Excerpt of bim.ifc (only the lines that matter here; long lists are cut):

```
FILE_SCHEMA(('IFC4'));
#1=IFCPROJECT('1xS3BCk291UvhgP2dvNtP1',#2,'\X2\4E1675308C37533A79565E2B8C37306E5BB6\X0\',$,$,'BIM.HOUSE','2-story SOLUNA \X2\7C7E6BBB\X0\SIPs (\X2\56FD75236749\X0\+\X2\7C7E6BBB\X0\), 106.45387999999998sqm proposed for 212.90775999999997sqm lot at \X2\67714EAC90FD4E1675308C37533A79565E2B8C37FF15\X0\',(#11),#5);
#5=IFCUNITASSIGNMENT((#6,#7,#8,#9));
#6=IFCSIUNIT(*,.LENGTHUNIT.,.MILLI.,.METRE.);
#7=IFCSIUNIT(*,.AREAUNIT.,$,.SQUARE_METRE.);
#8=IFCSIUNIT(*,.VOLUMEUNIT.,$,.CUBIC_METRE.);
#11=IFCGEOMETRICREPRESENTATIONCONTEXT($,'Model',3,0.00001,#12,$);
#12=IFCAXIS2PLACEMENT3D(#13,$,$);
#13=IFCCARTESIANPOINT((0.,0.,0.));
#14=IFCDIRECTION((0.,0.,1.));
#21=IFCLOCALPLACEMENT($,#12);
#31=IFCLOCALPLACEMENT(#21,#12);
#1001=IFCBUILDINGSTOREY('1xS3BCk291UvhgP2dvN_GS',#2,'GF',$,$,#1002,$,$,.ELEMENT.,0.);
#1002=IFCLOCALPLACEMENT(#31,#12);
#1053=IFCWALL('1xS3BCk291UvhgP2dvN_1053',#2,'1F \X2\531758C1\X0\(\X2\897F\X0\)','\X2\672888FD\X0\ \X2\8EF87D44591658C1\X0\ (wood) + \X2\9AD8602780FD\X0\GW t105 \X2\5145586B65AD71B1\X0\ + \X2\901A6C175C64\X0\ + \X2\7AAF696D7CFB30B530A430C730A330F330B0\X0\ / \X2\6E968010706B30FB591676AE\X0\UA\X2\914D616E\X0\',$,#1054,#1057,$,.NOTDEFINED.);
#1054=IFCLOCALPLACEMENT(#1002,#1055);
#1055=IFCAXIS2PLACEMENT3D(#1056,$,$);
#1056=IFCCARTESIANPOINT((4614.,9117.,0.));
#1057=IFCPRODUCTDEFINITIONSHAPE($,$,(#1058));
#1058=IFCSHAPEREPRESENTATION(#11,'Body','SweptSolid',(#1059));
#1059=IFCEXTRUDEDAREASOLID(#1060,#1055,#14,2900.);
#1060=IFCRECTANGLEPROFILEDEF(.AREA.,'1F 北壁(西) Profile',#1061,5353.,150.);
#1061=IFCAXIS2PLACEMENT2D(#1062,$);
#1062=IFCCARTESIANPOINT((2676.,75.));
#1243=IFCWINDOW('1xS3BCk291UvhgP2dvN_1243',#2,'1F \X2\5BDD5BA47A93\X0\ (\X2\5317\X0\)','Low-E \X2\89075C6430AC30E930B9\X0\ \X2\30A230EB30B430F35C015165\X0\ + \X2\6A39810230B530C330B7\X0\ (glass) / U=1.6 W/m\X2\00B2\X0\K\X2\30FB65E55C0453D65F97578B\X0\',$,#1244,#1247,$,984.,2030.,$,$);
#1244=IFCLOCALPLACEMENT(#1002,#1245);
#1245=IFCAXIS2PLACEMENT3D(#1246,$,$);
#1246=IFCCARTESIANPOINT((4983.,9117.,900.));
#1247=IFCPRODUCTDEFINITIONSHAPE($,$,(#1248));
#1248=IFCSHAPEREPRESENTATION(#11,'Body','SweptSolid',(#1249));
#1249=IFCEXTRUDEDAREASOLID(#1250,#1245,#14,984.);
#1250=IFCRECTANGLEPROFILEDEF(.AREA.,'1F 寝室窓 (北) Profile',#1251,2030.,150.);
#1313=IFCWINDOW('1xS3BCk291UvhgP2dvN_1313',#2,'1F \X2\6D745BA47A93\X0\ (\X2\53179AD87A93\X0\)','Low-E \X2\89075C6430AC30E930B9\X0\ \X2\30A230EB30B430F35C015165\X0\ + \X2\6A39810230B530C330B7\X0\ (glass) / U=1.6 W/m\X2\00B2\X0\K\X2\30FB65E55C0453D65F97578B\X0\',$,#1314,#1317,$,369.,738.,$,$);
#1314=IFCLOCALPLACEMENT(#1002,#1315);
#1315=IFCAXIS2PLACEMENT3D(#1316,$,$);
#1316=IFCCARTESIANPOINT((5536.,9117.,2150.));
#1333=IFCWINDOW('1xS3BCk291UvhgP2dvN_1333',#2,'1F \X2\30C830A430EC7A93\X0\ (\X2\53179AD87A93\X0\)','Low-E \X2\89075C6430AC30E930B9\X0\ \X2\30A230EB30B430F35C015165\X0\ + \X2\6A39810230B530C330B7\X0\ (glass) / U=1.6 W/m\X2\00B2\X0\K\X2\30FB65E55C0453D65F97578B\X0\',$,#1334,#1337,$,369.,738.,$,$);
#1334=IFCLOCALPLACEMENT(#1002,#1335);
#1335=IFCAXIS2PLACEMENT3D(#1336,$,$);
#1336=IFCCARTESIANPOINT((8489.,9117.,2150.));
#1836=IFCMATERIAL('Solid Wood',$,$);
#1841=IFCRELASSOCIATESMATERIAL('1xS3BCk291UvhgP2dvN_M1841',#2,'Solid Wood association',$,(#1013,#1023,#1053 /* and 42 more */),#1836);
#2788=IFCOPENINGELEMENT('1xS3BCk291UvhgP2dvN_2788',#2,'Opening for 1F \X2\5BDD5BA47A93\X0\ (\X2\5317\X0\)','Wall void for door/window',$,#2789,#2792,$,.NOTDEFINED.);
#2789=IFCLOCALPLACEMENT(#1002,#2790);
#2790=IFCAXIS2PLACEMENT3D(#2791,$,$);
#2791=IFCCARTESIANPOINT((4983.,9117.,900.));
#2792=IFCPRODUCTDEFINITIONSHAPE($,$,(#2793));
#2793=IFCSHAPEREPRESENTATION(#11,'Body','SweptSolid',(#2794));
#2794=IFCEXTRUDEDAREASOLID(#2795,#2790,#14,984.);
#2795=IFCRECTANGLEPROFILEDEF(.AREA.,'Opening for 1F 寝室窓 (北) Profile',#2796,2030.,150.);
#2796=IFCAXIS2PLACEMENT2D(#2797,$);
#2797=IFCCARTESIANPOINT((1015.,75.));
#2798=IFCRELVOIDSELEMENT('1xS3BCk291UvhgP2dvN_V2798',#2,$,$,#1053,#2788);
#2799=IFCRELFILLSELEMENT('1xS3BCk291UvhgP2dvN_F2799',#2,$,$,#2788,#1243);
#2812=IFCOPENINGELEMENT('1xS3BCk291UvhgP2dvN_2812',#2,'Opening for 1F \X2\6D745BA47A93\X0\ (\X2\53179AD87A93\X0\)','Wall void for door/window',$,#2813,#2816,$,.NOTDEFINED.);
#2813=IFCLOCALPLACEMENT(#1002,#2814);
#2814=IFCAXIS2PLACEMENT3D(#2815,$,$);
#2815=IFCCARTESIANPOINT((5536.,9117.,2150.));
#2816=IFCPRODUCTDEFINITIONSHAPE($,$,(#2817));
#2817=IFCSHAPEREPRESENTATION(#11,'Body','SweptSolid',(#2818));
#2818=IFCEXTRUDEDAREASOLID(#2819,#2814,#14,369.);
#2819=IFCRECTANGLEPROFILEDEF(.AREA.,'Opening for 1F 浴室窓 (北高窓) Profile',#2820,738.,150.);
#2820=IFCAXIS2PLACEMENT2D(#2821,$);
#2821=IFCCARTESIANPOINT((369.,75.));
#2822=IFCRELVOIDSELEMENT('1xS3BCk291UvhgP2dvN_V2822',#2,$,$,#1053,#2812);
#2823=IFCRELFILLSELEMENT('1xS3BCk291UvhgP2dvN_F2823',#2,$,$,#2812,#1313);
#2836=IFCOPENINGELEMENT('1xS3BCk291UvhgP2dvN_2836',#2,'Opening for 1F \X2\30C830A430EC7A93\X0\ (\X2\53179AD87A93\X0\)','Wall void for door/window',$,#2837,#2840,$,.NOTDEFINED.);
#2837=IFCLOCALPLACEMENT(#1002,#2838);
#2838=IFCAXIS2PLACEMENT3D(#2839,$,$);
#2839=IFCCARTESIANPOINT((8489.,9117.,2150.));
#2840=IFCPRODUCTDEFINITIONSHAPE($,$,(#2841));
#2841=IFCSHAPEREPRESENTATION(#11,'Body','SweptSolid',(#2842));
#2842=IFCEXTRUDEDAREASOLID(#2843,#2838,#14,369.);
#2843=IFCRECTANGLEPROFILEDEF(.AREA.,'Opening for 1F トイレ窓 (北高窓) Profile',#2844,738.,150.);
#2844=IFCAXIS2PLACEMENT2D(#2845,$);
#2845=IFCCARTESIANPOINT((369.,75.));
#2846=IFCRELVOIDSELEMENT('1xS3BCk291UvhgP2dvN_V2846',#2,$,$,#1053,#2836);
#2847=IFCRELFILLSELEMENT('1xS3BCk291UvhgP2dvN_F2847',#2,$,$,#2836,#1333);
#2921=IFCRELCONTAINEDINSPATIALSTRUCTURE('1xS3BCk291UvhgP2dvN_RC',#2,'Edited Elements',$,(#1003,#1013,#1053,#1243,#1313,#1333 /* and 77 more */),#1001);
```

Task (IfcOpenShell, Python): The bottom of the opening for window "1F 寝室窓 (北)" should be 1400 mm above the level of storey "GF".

```python
import numpy as np
import ifcopenshell
import ifcopenshell.api.geometry
import ifcopenshell.geom
import ifcopenshell.util.element
import ifcopenshell.util.placement
import ifcopenshell.util.shape
import ifcopenshell.util.unit

model = ifcopenshell.open("bim.ifc")
unit_scale = ifcopenshell.util.unit.calculate_unit_scale(model)

window = model.by_guid("1xS3BCk291UvhgP2dvN_1243")
opening = window.FillsVoids[0].RelatingOpeningElement
storey = ifcopenshell.util.element.get_container(window, ifc_class="IfcBuildingStorey")
level = ifcopenshell.util.placement.get_local_placement(storey.ObjectPlacement)[2, 3]

# The opening's origin need not be at the sill, so measure its lowest point.
shape = ifcopenshell.geom.create_shape(ifcopenshell.geom.settings(), opening)
bottom = ifcopenshell.util.shape.get_shape_bottom_elevation(shape, shape.geometry) / unit_scale
dz = level + 1400.0 - bottom

shift = np.array([0.0, 0.0, dz])
# The window is not placed relative to its opening, so move both.
for product in (opening, window):
    matrix = ifcopenshell.util.placement.get_local_placement(product.ObjectPlacement)
    matrix[:3, 3] += shift
    ifcopenshell.api.geometry.edit_object_placement(model, product=product, matrix=matrix, is_si=False)

print(f"moved by {dz * unit_scale:+.3f} m")

model.write("bim_v2.ifc")
```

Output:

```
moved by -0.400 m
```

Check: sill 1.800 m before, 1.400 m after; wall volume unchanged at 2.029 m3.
